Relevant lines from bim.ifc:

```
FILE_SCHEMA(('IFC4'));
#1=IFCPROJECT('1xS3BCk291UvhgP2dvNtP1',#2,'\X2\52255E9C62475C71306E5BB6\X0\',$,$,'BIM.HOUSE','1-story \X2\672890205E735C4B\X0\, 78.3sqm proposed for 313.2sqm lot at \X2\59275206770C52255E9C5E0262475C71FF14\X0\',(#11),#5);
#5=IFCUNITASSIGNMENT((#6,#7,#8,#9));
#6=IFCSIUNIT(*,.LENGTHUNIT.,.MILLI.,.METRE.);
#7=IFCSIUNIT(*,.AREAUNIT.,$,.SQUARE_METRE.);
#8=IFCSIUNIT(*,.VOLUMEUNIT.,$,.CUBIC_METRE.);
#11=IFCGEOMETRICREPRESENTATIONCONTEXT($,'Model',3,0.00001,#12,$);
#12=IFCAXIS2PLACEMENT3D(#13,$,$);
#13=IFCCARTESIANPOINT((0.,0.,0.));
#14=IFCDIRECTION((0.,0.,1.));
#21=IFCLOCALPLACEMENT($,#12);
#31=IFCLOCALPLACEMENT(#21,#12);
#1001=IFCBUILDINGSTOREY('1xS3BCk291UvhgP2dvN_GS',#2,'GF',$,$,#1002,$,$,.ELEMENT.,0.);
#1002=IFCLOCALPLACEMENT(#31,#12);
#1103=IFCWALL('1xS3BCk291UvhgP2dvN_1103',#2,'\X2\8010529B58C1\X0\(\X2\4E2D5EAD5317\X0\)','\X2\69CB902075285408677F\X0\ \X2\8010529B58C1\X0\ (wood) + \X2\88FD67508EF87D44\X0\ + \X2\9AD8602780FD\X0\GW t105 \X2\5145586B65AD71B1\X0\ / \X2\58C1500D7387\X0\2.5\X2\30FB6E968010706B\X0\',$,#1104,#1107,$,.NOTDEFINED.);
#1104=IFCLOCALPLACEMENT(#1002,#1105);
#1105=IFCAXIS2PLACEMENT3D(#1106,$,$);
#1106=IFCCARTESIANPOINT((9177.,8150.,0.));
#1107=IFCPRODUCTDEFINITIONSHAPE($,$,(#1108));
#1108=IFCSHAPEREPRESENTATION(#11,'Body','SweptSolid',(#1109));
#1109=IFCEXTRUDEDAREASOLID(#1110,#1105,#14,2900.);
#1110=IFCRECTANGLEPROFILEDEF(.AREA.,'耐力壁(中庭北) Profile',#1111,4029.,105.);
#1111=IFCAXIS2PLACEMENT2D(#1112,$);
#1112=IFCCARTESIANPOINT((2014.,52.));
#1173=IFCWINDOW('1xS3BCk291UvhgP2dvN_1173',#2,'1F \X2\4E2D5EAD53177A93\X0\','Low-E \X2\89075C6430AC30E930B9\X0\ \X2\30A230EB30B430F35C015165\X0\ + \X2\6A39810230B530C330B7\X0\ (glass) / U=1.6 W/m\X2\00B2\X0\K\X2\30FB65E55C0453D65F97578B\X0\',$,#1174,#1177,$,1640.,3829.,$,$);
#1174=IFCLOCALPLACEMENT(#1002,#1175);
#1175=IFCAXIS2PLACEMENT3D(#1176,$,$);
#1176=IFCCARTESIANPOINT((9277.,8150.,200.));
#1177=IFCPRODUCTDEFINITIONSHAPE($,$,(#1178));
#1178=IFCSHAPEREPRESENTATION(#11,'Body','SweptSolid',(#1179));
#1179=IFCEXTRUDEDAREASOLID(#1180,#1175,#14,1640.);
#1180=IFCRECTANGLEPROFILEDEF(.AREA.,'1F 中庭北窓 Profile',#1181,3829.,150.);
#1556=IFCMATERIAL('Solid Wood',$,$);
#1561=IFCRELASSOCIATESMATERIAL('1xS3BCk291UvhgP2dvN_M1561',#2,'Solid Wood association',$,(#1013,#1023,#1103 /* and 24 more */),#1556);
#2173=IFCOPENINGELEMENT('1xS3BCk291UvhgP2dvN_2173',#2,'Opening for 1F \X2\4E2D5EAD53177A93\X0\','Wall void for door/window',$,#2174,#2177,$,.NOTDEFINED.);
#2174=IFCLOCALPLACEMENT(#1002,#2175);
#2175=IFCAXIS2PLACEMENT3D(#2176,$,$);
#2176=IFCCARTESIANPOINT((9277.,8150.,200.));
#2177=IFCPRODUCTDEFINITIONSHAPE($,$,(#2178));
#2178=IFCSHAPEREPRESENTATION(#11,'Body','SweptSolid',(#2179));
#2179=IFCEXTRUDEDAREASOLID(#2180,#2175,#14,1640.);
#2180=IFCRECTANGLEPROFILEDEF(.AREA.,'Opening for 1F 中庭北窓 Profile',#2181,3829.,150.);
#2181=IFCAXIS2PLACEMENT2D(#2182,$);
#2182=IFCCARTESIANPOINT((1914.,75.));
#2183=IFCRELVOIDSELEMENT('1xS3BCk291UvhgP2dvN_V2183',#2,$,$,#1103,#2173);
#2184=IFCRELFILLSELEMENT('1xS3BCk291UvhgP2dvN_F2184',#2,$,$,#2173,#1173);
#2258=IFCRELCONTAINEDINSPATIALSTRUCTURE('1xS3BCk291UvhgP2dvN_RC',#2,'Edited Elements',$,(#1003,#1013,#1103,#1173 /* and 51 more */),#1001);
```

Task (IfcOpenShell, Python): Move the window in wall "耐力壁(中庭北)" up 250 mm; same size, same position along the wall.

```python
import numpy as np
import ifcopenshell
import ifcopenshell.api.geometry
import ifcopenshell.util.placement
import ifcopenshell.util.unit

model = ifcopenshell.open("bim.ifc")
unit_scale = ifcopenshell.util.unit.calculate_unit_scale(model)

window = model.by_guid("1xS3BCk291UvhgP2dvN_1173")
opening = window.FillsVoids[0].RelatingOpeningElement
dz = 0.25 / unit_scale

shift = np.array([0.0, 0.0, dz])
# The window is not placed relative to its opening, so move both.
for product in (opening, window):
    matrix = ifcopenshell.util.placement.get_local_placement(product.ObjectPlacement)
    matrix[:3, 3] += shift
    ifcopenshell.api.geometry.edit_object_placement(model, product=product, matrix=matrix, is_si=False)

print(f"moved by {dz * unit_scale:+.3f} m")

model.write("bim_v2.ifc")
```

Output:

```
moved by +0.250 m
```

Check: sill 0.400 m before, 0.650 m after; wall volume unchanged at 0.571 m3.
